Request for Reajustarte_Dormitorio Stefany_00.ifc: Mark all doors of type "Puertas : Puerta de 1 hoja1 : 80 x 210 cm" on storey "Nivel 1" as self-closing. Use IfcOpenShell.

First a look at what the model holds.

```python
import ifcopenshell
import ifcopenshell.util.element

model = ifcopenshell.open("Reajustarte_Dormitorio Stefany_00.ifc")
print(model.schema)
storey = next(s for s in model.by_type("IfcBuildingStorey") if s.Name == "Nivel 1")
doors = [e for e in ifcopenshell.util.element.get_decomposition(storey) if e.is_a("IfcDoor")]
seen = {}
for e in doors:
    element_type = ifcopenshell.util.element.get_type(e)
    key = (element_type.Name if element_type != e and element_type else None, ifcopenshell.util.element.get_pset(e, "Pset_DoorCommon", "SelfClosing"))
    seen[key] = seen.get(key, 0) + 1
for (name, value), count in sorted(seen.items(), key=str):
    print(count, "x", name, "|", value)
```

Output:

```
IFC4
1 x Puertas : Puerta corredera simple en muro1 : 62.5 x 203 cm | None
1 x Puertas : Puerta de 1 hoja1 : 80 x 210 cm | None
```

```python
import ifcopenshell
import ifcopenshell.api.pset
import ifcopenshell.util.element

model = ifcopenshell.open("Reajustarte_Dormitorio Stefany_00.ifc")

storey = next(s for s in model.by_type("IfcBuildingStorey") if s.Name == "Nivel 1")
doors = [e for e in ifcopenshell.util.element.get_decomposition(storey) if e.is_a("IfcDoor")]

count = 0
for e in doors:
    element_type = ifcopenshell.util.element.get_type(e)
    if element_type in (None, e) or element_type.Name != "Puertas : Puerta de 1 hoja1 : 80 x 210 cm":
        continue
    # add_pset returns the element's existing set when there is one.
    pset = ifcopenshell.api.pset.add_pset(model, product=e, name="Pset_DoorCommon")
    ifcopenshell.api.pset.edit_pset(model, pset=pset, properties={"SelfClosing": True})
    count += 1

print(count, "doors updated")

model.write("Reajustarte_Dormitorio Stefany_00_edited.ifc")
```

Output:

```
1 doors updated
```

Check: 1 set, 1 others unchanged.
